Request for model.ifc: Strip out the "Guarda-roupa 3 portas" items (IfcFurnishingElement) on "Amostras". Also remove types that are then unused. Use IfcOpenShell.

First a look at what the model holds.

```python
import ifcopenshell
import ifcopenshell.util.element

model = ifcopenshell.open("model.ifc")
print(model.schema)
storey = next(s for s in model.by_type("IfcBuildingStorey") if s.Name == "Amostras")
furniture = [e for e in ifcopenshell.util.element.get_decomposition(storey) if e.is_a("IfcFurnishingElement")]
seen = {}
for e in furniture:
    element_type = ifcopenshell.util.element.get_type(e)
    name = element_type.Name if element_type not in (None, e) else None
    seen[name] = seen.get(name, 0) + 1
for name, count in sorted(seen.items(), key=str):
    print(count, "x", name)
```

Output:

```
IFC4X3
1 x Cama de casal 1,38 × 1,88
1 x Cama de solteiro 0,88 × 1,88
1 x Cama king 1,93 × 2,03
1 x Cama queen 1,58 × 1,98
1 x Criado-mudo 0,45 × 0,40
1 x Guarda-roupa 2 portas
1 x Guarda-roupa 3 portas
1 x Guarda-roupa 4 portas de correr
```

```python
import ifcopenshell
import ifcopenshell.api.root
import ifcopenshell.util.element

model = ifcopenshell.open("model.ifc")

storey = next(s for s in model.by_type("IfcBuildingStorey") if s.Name == "Amostras")
furniture = [e for e in ifcopenshell.util.element.get_decomposition(storey) if e.is_a("IfcFurnishingElement")]
targets = [e for e in furniture if (t := ifcopenshell.util.element.get_type(e)) not in (None, e) and t.Name == "Guarda-roupa 3 portas"]
types = {ifcopenshell.util.element.get_type(e) for e in targets} - {None, *targets}

for e in targets:
    ifcopenshell.api.root.remove_product(model, product=e)
print(len(targets), "removed")

unused = [t for t in types if not ifcopenshell.util.element.get_types(t)]
for t in unused:
    ifcopenshell.api.root.remove_product(model, product=t)
print(len(unused), "unused types removed")

model.write("model-out.ifc")
```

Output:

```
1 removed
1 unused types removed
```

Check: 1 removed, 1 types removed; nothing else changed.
